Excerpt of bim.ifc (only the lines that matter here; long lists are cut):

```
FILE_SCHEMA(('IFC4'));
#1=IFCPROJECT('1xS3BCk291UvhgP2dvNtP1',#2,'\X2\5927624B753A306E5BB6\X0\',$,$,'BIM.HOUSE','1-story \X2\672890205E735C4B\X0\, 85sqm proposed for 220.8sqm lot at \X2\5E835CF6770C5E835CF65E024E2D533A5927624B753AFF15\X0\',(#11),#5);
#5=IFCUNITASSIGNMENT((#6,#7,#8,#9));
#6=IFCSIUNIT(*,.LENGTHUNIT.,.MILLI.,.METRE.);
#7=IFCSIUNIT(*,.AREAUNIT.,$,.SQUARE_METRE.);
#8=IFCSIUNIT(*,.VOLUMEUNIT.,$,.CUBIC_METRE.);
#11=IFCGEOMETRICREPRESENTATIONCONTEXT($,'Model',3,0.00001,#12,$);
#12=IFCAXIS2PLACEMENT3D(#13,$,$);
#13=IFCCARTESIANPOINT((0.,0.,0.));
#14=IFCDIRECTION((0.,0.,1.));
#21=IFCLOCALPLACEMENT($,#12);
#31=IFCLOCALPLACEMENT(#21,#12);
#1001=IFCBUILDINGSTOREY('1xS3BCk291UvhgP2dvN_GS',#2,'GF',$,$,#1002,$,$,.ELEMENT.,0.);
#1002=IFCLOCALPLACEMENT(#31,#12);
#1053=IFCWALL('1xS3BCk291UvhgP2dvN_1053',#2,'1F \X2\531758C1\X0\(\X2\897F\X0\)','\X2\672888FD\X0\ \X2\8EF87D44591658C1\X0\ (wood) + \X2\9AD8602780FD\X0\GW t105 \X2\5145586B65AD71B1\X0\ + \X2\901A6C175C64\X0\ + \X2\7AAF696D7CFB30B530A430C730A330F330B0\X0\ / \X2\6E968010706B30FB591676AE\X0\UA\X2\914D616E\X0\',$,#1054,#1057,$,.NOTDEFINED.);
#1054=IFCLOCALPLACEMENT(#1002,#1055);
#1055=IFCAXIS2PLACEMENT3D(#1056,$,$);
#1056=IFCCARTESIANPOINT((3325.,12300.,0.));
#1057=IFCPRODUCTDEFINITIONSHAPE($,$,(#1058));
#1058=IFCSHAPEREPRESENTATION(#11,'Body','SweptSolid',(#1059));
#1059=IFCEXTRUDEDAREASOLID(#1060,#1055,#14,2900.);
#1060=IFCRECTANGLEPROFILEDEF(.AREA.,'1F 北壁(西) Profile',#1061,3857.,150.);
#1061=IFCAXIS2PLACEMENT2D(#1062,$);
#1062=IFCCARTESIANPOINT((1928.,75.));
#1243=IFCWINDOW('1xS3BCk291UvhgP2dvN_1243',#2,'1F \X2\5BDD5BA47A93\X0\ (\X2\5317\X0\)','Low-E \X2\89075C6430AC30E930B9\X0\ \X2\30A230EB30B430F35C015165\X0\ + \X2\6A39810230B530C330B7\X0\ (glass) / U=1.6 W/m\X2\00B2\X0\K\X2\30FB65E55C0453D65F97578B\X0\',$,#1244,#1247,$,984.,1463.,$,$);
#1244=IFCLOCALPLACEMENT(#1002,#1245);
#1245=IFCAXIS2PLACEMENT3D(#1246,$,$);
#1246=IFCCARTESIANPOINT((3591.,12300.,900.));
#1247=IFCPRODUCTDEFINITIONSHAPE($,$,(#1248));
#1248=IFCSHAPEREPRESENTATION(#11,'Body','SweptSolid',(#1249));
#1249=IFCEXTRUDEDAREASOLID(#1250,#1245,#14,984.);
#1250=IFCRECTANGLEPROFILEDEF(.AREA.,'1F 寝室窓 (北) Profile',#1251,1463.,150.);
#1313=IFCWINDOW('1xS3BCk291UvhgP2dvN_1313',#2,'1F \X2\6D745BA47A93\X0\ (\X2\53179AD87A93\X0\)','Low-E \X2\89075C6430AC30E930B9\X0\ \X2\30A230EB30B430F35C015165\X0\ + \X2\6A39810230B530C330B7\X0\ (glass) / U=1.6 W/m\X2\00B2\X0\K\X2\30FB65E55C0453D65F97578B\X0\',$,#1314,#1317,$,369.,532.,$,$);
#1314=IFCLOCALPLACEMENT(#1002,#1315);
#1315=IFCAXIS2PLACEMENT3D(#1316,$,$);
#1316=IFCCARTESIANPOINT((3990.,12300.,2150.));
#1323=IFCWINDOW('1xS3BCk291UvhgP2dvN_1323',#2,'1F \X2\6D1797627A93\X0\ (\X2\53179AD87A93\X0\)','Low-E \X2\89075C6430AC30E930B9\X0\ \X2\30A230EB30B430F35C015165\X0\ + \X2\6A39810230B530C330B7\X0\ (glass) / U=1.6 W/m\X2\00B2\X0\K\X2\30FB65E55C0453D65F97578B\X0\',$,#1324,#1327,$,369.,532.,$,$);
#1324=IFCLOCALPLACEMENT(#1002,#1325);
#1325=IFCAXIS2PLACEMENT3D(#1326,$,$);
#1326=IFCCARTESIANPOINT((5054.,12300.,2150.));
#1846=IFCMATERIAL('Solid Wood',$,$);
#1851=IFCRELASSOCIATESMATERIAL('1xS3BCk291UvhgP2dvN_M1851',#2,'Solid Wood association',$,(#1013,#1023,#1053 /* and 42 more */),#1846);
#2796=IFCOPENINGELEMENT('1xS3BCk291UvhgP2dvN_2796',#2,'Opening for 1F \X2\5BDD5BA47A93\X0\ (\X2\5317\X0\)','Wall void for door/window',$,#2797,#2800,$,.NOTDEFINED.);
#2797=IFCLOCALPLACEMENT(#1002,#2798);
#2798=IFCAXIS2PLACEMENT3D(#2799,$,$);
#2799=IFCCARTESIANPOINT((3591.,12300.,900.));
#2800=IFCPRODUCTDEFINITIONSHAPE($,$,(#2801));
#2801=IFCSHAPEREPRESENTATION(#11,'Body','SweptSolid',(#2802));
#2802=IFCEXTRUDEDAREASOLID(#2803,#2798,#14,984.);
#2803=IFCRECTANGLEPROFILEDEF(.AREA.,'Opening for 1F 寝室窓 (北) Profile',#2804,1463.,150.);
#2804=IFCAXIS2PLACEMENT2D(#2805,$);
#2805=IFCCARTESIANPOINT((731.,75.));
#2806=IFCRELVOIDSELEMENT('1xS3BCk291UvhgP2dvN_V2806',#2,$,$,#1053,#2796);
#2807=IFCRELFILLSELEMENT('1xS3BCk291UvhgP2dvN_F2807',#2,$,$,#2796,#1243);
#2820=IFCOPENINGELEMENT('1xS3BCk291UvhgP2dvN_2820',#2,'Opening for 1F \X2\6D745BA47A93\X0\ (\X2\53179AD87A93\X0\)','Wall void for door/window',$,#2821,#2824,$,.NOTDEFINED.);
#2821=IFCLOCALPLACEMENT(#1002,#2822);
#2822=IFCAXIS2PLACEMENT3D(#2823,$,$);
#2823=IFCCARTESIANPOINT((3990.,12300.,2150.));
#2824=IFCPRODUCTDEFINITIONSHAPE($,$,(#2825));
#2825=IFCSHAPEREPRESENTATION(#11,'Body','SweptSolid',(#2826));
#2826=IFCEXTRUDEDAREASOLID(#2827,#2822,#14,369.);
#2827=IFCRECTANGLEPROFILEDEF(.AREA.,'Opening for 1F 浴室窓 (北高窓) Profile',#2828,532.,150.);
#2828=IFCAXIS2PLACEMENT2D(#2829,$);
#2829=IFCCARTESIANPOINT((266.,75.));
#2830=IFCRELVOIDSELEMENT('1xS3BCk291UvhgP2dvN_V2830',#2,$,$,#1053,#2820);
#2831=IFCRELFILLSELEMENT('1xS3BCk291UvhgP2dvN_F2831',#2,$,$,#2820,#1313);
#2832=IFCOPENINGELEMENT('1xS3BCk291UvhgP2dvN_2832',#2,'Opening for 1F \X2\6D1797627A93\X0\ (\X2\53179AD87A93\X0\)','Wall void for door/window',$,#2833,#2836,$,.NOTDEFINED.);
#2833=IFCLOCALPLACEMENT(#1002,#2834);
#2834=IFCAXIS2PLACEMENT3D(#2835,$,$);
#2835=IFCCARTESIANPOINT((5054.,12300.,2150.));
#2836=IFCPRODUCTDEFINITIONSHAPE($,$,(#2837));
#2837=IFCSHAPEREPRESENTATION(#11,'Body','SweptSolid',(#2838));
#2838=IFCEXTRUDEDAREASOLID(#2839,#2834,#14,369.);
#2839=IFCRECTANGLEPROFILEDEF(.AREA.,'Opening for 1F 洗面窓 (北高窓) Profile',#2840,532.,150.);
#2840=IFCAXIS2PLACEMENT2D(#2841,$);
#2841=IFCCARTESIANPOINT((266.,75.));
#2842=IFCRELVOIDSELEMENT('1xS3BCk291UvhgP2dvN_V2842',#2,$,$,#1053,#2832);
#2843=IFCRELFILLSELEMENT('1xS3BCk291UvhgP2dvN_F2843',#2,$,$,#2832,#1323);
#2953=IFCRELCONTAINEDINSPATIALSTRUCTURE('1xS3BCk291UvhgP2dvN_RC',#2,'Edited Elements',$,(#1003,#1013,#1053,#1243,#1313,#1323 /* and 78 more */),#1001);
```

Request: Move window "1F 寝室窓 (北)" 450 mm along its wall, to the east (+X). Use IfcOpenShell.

```python
import ifcopenshell
import ifcopenshell.api.geometry
import ifcopenshell.util.placement
import ifcopenshell.util.unit

model = ifcopenshell.open("bim.ifc")
unit_scale = ifcopenshell.util.unit.calculate_unit_scale(model)

window = model.by_guid("1xS3BCk291UvhgP2dvN_1243")
opening = window.FillsVoids[0].RelatingOpeningElement
wall = opening.VoidsElements[0].RelatingBuildingElement

wall_matrix = ifcopenshell.util.placement.get_local_placement(wall.ObjectPlacement)
shift = wall_matrix[:3, 0] * 0.45 / unit_scale
before = ifcopenshell.util.placement.get_local_placement(window.ObjectPlacement)[:3, 3].copy()

# The window is not placed relative to its opening, so move both.
for product in (opening, window):
    matrix = ifcopenshell.util.placement.get_local_placement(product.ObjectPlacement)
    matrix[:3, 3] += shift
    ifcopenshell.api.geometry.edit_object_placement(model, product=product, matrix=matrix, is_si=False)

after = ifcopenshell.util.placement.get_local_placement(window.ObjectPlacement)[:3, 3]
print("window moved by", (after - before).round(3) + 0.0)

model.write("bim_v2.ifc")
```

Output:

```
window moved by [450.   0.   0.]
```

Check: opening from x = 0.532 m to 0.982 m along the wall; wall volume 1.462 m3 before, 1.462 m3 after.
